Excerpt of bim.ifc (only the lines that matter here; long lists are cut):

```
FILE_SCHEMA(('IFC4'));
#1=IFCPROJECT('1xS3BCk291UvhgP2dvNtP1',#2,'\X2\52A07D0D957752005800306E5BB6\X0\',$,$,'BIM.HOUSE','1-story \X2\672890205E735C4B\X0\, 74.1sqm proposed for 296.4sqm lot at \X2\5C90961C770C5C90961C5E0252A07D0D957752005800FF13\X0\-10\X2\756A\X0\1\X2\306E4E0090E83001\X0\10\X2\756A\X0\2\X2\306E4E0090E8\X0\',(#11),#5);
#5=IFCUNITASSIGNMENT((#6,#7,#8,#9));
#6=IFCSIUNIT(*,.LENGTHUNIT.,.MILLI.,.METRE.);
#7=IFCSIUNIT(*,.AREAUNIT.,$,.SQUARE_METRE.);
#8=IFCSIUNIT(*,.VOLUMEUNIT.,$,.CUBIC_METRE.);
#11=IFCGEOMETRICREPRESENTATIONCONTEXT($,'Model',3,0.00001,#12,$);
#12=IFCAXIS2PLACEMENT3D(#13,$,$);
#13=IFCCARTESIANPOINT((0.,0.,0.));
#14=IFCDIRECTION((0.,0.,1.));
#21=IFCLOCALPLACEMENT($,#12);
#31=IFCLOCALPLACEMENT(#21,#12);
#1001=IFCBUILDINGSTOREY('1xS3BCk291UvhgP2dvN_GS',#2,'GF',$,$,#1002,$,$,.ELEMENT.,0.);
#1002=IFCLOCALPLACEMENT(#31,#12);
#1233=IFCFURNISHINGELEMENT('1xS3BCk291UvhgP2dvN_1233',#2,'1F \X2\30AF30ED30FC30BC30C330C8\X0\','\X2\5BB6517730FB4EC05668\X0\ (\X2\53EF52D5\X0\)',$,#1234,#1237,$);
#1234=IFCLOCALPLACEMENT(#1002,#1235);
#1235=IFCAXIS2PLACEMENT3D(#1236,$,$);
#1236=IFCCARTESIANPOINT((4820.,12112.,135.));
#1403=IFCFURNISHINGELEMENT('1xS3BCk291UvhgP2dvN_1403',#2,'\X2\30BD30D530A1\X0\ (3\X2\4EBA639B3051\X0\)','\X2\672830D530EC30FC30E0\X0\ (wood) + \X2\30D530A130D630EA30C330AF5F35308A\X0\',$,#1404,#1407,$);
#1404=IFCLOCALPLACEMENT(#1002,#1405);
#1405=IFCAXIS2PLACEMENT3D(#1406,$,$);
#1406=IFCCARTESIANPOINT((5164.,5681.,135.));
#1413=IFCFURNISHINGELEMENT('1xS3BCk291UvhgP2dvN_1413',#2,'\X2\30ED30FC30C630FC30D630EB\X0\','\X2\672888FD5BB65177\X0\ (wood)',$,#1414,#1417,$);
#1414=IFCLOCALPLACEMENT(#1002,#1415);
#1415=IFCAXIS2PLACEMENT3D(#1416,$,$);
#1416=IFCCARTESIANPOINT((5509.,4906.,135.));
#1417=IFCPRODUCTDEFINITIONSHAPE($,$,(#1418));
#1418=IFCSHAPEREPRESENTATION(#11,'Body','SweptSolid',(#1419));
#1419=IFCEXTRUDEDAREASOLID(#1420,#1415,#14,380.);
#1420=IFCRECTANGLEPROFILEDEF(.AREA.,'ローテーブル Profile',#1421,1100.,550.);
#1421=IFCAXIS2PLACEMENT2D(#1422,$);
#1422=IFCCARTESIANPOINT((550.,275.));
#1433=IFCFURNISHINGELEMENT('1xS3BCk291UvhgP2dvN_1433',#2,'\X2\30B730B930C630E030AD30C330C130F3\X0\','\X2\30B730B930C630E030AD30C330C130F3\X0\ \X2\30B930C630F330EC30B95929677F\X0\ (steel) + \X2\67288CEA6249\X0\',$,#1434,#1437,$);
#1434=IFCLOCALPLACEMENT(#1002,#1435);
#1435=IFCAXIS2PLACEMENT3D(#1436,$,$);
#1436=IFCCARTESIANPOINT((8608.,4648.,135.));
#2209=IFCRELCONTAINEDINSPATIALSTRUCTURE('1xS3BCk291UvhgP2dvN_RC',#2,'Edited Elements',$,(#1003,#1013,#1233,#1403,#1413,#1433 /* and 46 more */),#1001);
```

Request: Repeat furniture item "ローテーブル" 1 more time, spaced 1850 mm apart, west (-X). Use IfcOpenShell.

```python
import numpy as np
import ifcopenshell
import ifcopenshell.api.geometry
import ifcopenshell.api.root
import ifcopenshell.util.element
import ifcopenshell.util.placement

model = ifcopenshell.open("bim.ifc")


def reuse_history(source, copy):
    """copy_class also copies each property set's owner history, people and application; keep the originals."""
    for rel in copy.IsDefinedBy:
        if rel.is_a("IfcRelDefinesByProperties") and (history := rel.RelatingPropertyDefinition.OwnerHistory):
            rel.RelatingPropertyDefinition.OwnerHistory = source.OwnerHistory
            ifcopenshell.util.element.remove_deep2(model, history)


source = model.by_id(1413)
base = ifcopenshell.util.placement.get_local_placement(source.ObjectPlacement)
step = np.array([-1.0, 0.0, 0.0]) * 1850.0

for i in range(1, 2):
    copy = ifcopenshell.api.root.copy_class(model, product=source)
    copy.Representation = ifcopenshell.util.element.copy_deep(
        model, source.Representation, exclude=["IfcGeometricRepresentationContext", "IfcRepresentationMap"]
    )
    reuse_history(source, copy)
    matrix = base.copy()
    matrix[:3, 3] += i * step
    print("added at", matrix[:3, 3].round(3) + 0.0)
    ifcopenshell.api.geometry.edit_object_placement(model, product=copy, matrix=matrix, is_si=False)

model.write("bim-out.ifc")
```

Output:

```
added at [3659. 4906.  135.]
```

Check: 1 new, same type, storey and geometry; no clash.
